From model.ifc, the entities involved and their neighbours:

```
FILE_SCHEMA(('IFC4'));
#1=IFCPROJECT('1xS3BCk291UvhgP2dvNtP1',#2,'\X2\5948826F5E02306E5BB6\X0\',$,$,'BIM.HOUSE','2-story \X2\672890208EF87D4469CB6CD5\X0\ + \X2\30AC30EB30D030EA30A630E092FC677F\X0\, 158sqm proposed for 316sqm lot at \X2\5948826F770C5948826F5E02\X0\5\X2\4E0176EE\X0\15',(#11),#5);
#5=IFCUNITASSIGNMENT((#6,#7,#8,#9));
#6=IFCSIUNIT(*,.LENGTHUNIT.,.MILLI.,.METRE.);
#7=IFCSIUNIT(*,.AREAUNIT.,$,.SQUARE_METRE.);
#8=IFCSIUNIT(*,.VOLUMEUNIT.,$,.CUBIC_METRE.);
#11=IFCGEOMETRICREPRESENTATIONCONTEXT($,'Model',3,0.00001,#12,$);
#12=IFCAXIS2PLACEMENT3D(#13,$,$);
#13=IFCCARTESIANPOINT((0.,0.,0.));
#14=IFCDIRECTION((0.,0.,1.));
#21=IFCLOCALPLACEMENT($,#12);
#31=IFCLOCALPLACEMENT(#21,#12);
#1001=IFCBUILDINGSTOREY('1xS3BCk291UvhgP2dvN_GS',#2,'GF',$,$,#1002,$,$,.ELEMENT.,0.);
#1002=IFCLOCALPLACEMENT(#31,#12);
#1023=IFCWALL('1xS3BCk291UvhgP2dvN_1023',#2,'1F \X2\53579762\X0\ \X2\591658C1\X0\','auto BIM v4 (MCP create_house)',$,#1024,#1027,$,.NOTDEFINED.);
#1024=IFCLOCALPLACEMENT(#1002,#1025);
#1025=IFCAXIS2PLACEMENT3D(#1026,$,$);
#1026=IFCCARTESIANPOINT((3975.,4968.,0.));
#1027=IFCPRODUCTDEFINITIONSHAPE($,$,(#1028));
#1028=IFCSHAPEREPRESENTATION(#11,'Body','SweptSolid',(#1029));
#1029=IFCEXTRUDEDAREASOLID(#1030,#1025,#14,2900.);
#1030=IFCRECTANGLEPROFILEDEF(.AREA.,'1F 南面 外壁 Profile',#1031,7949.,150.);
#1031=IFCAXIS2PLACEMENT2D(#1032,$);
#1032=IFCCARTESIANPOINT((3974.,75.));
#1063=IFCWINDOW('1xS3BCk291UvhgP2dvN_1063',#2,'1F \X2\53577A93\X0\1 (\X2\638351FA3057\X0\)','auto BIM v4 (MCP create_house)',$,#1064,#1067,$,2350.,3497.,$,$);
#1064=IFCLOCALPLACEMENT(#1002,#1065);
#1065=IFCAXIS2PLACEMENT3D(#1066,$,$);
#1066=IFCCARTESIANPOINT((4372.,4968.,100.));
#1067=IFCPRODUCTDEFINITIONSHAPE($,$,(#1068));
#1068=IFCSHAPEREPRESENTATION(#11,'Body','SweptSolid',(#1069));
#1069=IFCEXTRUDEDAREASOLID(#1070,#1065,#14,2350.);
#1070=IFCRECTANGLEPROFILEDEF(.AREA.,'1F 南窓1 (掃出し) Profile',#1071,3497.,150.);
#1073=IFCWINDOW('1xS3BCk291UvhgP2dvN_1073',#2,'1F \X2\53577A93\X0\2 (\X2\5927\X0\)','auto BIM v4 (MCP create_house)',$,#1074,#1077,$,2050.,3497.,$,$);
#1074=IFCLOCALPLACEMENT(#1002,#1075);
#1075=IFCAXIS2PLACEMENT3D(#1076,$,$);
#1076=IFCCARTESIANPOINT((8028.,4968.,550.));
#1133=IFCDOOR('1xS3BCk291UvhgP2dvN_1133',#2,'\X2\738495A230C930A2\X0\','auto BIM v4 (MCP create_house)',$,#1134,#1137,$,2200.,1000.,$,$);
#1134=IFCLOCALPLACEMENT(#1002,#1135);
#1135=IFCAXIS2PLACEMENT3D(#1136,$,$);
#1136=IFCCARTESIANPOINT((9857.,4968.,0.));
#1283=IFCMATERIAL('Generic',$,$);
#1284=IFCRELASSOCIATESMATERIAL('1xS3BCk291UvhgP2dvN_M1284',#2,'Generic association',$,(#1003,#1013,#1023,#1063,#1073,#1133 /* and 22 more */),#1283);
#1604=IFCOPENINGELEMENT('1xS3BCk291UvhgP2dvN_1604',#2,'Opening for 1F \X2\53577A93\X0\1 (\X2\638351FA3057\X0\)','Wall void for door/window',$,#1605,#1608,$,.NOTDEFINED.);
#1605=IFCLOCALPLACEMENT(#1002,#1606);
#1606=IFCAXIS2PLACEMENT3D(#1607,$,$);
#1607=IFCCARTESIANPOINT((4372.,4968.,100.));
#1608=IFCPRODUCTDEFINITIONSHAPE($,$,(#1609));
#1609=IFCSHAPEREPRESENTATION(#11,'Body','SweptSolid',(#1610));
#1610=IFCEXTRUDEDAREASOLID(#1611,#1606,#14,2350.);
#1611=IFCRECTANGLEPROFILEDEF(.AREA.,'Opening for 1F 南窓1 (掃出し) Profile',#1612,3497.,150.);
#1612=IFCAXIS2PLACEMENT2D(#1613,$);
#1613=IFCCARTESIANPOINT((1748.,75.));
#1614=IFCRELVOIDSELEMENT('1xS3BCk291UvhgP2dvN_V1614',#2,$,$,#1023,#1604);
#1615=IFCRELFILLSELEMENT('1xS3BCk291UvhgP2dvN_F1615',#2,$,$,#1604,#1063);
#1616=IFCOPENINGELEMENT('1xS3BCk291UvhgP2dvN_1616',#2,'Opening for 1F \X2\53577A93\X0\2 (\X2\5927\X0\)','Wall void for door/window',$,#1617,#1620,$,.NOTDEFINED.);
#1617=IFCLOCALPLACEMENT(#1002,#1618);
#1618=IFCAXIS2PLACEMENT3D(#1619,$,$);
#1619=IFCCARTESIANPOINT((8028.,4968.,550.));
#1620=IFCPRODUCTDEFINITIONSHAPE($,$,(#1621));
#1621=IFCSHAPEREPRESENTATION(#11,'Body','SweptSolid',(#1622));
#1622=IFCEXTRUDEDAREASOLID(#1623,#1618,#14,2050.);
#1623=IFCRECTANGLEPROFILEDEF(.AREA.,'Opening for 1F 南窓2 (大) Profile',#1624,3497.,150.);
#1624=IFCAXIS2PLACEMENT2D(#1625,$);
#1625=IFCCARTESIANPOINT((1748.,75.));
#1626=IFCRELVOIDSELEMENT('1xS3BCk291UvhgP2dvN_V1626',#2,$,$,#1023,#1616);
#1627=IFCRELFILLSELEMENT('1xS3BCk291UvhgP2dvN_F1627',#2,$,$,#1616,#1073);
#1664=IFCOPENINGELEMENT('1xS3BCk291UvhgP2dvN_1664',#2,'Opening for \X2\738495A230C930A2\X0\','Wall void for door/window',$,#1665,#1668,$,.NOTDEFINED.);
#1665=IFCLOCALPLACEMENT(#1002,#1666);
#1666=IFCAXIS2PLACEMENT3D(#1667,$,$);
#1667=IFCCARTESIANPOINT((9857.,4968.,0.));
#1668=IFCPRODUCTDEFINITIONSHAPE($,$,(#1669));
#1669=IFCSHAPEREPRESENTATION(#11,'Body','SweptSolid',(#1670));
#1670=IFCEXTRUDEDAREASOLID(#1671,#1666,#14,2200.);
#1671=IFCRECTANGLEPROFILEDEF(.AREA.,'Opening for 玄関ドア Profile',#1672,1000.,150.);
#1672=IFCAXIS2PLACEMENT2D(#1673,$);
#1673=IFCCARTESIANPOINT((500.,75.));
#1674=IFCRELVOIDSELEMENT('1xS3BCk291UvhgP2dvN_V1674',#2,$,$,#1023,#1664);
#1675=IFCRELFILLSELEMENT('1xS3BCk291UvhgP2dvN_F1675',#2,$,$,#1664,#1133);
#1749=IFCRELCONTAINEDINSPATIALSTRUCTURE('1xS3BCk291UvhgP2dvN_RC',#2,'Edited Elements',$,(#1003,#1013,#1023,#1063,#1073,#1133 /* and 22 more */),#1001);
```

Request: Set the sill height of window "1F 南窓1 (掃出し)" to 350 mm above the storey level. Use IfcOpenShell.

```python
import numpy as np
import ifcopenshell
import ifcopenshell.api.geometry
import ifcopenshell.geom
import ifcopenshell.util.element
import ifcopenshell.util.placement
import ifcopenshell.util.shape
import ifcopenshell.util.unit

model = ifcopenshell.open("model.ifc")
unit_scale = ifcopenshell.util.unit.calculate_unit_scale(model)

window = model.by_guid("1xS3BCk291UvhgP2dvN_1063")
opening = window.FillsVoids[0].RelatingOpeningElement
storey = ifcopenshell.util.element.get_container(window, ifc_class="IfcBuildingStorey")
level = ifcopenshell.util.placement.get_local_placement(storey.ObjectPlacement)[2, 3]

# The opening's origin need not be at the sill, so measure its lowest point.
shape = ifcopenshell.geom.create_shape(ifcopenshell.geom.settings(), opening)
bottom = ifcopenshell.util.shape.get_shape_bottom_elevation(shape, shape.geometry) / unit_scale
dz = level + 350.0 - bottom

shift = np.array([0.0, 0.0, dz])
# The window is not placed relative to its opening, so move both.
for product in (opening, window):
    matrix = ifcopenshell.util.placement.get_local_placement(product.ObjectPlacement)
    matrix[:3, 3] += shift
    ifcopenshell.api.geometry.edit_object_placement(model, product=product, matrix=matrix, is_si=False)

print(f"moved by {dz * unit_scale:+.3f} m")

model.write("model_rev.ifc")
```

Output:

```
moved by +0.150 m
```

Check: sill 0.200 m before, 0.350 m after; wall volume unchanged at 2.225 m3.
